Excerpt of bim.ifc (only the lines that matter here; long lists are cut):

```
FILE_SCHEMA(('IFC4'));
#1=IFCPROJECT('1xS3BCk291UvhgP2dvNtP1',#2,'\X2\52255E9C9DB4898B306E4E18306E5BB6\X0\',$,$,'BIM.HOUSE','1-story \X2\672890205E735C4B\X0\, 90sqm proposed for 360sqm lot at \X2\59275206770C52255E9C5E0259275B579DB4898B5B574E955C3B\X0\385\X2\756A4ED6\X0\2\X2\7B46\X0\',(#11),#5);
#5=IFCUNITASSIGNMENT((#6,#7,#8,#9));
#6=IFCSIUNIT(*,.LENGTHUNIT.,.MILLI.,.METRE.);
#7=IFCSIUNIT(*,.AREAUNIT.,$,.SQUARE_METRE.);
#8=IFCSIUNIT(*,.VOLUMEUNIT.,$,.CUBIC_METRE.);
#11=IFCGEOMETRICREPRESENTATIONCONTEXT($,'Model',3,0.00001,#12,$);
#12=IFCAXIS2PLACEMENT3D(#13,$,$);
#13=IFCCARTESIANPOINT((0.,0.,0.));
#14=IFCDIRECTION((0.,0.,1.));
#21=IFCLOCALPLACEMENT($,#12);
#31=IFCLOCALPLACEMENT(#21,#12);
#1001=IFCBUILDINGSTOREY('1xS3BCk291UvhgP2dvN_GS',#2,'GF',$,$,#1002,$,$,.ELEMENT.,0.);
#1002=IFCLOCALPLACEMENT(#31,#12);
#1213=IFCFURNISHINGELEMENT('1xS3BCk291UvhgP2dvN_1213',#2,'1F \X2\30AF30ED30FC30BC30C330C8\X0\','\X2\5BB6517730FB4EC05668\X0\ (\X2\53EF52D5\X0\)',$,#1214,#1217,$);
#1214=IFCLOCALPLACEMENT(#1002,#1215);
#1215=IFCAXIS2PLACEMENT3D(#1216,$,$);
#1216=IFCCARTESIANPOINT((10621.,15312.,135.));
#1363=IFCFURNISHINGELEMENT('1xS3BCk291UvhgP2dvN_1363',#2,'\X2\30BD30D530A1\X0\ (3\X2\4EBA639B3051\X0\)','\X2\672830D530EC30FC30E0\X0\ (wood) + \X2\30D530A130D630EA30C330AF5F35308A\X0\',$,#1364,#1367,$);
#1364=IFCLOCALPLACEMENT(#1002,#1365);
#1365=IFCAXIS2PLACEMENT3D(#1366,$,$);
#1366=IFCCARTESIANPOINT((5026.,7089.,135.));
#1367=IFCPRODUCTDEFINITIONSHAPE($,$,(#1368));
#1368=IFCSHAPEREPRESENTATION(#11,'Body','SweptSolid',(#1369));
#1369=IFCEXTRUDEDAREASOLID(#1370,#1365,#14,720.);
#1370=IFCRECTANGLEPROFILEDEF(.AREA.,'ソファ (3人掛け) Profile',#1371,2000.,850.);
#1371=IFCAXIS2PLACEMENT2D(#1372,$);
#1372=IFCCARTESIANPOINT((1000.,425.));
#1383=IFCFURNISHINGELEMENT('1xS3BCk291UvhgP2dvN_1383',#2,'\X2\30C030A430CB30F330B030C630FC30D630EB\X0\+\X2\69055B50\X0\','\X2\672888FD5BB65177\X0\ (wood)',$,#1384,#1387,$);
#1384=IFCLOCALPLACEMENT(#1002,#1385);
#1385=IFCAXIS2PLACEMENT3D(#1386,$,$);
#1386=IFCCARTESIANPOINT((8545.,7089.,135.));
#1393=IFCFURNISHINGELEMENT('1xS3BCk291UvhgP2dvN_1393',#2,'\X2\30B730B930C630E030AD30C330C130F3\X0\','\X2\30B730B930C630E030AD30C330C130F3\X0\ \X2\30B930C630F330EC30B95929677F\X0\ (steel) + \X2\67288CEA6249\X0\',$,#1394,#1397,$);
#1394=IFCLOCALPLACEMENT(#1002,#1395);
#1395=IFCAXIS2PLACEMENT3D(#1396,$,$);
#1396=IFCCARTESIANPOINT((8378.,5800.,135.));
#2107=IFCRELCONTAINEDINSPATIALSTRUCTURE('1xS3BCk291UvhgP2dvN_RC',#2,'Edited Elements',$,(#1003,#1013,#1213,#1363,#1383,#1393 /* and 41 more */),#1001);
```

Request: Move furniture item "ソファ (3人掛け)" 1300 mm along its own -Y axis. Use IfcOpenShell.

```python
import ifcopenshell
import ifcopenshell.api.geometry
import ifcopenshell.util.placement
import ifcopenshell.util.unit

model = ifcopenshell.open("bim.ifc")
unit_scale = ifcopenshell.util.unit.calculate_unit_scale(model)

item = model.by_guid("1xS3BCk291UvhgP2dvN_1363")
matrix = ifcopenshell.util.placement.get_local_placement(item.ObjectPlacement)
matrix[:3, 3] -= matrix[:3, 1] * 1.3 / unit_scale
ifcopenshell.api.geometry.edit_object_placement(model, product=item, matrix=matrix, is_si=False)

print(ifcopenshell.util.placement.get_local_placement(item.ObjectPlacement).round(3) + 0.0)

model.write("bim_updated.ifc")
```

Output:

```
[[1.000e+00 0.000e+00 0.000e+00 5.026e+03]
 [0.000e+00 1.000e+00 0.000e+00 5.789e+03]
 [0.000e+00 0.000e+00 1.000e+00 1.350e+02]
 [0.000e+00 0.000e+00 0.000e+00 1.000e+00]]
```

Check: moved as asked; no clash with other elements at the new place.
